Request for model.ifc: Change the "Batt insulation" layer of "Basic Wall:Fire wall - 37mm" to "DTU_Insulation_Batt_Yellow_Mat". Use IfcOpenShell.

First a look at what the model holds.

```python
import ifcopenshell
import ifcopenshell.util.element

model = ifcopenshell.open("model.ifc")
print(model.schema)
for layer_set in model.by_type("IfcMaterialLayerSet"):
    if layer_set.LayerSetName == "Basic Wall:Fire wall - 37mm":
        for layer in layer_set.MaterialLayers:
            print(layer.id(), layer.Material and layer.Material.Name, layer.LayerThickness, sep=" | ")
        print(len(ifcopenshell.util.element.get_elements_by_material(model, layer_set)), "elements and types use it")
print(sorted(m.Name for m in model.by_type("IfcMaterial") if m.Name)[:60])
```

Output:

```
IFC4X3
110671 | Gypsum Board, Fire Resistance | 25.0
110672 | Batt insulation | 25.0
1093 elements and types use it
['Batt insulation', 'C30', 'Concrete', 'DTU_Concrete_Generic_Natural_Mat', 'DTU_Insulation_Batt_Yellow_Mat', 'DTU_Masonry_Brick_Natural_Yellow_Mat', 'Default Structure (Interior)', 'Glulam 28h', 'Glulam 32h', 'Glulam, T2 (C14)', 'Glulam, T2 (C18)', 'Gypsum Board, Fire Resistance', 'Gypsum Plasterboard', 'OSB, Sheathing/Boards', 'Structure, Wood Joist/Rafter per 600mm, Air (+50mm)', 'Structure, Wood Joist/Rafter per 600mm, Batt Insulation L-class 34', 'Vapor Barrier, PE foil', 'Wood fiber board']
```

```python
import ifcopenshell
import ifcopenshell.api.material

model = ifcopenshell.open("model.ifc")

layer_set = next(s for s in model.by_type("IfcMaterialLayerSet") if s.LayerSetName == "Basic Wall:Fire wall - 37mm")
layer = next(l for l in layer_set.MaterialLayers if l.Material and l.Material.Name == "Batt insulation")
material = next(m for m in model.by_type("IfcMaterial") if m.Name == "DTU_Insulation_Batt_Yellow_Mat")

# Point this one layer at the other material; renaming the old one would change it everywhere.
ifcopenshell.api.material.edit_layer(model, layer=layer, attributes={"Name": material.Name}, material=material)

print([l.Material.Name if l.Material else None for l in layer_set.MaterialLayers])

model.write("model_v2.ifc")
```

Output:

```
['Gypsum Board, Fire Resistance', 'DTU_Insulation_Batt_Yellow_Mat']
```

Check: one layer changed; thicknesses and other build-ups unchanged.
